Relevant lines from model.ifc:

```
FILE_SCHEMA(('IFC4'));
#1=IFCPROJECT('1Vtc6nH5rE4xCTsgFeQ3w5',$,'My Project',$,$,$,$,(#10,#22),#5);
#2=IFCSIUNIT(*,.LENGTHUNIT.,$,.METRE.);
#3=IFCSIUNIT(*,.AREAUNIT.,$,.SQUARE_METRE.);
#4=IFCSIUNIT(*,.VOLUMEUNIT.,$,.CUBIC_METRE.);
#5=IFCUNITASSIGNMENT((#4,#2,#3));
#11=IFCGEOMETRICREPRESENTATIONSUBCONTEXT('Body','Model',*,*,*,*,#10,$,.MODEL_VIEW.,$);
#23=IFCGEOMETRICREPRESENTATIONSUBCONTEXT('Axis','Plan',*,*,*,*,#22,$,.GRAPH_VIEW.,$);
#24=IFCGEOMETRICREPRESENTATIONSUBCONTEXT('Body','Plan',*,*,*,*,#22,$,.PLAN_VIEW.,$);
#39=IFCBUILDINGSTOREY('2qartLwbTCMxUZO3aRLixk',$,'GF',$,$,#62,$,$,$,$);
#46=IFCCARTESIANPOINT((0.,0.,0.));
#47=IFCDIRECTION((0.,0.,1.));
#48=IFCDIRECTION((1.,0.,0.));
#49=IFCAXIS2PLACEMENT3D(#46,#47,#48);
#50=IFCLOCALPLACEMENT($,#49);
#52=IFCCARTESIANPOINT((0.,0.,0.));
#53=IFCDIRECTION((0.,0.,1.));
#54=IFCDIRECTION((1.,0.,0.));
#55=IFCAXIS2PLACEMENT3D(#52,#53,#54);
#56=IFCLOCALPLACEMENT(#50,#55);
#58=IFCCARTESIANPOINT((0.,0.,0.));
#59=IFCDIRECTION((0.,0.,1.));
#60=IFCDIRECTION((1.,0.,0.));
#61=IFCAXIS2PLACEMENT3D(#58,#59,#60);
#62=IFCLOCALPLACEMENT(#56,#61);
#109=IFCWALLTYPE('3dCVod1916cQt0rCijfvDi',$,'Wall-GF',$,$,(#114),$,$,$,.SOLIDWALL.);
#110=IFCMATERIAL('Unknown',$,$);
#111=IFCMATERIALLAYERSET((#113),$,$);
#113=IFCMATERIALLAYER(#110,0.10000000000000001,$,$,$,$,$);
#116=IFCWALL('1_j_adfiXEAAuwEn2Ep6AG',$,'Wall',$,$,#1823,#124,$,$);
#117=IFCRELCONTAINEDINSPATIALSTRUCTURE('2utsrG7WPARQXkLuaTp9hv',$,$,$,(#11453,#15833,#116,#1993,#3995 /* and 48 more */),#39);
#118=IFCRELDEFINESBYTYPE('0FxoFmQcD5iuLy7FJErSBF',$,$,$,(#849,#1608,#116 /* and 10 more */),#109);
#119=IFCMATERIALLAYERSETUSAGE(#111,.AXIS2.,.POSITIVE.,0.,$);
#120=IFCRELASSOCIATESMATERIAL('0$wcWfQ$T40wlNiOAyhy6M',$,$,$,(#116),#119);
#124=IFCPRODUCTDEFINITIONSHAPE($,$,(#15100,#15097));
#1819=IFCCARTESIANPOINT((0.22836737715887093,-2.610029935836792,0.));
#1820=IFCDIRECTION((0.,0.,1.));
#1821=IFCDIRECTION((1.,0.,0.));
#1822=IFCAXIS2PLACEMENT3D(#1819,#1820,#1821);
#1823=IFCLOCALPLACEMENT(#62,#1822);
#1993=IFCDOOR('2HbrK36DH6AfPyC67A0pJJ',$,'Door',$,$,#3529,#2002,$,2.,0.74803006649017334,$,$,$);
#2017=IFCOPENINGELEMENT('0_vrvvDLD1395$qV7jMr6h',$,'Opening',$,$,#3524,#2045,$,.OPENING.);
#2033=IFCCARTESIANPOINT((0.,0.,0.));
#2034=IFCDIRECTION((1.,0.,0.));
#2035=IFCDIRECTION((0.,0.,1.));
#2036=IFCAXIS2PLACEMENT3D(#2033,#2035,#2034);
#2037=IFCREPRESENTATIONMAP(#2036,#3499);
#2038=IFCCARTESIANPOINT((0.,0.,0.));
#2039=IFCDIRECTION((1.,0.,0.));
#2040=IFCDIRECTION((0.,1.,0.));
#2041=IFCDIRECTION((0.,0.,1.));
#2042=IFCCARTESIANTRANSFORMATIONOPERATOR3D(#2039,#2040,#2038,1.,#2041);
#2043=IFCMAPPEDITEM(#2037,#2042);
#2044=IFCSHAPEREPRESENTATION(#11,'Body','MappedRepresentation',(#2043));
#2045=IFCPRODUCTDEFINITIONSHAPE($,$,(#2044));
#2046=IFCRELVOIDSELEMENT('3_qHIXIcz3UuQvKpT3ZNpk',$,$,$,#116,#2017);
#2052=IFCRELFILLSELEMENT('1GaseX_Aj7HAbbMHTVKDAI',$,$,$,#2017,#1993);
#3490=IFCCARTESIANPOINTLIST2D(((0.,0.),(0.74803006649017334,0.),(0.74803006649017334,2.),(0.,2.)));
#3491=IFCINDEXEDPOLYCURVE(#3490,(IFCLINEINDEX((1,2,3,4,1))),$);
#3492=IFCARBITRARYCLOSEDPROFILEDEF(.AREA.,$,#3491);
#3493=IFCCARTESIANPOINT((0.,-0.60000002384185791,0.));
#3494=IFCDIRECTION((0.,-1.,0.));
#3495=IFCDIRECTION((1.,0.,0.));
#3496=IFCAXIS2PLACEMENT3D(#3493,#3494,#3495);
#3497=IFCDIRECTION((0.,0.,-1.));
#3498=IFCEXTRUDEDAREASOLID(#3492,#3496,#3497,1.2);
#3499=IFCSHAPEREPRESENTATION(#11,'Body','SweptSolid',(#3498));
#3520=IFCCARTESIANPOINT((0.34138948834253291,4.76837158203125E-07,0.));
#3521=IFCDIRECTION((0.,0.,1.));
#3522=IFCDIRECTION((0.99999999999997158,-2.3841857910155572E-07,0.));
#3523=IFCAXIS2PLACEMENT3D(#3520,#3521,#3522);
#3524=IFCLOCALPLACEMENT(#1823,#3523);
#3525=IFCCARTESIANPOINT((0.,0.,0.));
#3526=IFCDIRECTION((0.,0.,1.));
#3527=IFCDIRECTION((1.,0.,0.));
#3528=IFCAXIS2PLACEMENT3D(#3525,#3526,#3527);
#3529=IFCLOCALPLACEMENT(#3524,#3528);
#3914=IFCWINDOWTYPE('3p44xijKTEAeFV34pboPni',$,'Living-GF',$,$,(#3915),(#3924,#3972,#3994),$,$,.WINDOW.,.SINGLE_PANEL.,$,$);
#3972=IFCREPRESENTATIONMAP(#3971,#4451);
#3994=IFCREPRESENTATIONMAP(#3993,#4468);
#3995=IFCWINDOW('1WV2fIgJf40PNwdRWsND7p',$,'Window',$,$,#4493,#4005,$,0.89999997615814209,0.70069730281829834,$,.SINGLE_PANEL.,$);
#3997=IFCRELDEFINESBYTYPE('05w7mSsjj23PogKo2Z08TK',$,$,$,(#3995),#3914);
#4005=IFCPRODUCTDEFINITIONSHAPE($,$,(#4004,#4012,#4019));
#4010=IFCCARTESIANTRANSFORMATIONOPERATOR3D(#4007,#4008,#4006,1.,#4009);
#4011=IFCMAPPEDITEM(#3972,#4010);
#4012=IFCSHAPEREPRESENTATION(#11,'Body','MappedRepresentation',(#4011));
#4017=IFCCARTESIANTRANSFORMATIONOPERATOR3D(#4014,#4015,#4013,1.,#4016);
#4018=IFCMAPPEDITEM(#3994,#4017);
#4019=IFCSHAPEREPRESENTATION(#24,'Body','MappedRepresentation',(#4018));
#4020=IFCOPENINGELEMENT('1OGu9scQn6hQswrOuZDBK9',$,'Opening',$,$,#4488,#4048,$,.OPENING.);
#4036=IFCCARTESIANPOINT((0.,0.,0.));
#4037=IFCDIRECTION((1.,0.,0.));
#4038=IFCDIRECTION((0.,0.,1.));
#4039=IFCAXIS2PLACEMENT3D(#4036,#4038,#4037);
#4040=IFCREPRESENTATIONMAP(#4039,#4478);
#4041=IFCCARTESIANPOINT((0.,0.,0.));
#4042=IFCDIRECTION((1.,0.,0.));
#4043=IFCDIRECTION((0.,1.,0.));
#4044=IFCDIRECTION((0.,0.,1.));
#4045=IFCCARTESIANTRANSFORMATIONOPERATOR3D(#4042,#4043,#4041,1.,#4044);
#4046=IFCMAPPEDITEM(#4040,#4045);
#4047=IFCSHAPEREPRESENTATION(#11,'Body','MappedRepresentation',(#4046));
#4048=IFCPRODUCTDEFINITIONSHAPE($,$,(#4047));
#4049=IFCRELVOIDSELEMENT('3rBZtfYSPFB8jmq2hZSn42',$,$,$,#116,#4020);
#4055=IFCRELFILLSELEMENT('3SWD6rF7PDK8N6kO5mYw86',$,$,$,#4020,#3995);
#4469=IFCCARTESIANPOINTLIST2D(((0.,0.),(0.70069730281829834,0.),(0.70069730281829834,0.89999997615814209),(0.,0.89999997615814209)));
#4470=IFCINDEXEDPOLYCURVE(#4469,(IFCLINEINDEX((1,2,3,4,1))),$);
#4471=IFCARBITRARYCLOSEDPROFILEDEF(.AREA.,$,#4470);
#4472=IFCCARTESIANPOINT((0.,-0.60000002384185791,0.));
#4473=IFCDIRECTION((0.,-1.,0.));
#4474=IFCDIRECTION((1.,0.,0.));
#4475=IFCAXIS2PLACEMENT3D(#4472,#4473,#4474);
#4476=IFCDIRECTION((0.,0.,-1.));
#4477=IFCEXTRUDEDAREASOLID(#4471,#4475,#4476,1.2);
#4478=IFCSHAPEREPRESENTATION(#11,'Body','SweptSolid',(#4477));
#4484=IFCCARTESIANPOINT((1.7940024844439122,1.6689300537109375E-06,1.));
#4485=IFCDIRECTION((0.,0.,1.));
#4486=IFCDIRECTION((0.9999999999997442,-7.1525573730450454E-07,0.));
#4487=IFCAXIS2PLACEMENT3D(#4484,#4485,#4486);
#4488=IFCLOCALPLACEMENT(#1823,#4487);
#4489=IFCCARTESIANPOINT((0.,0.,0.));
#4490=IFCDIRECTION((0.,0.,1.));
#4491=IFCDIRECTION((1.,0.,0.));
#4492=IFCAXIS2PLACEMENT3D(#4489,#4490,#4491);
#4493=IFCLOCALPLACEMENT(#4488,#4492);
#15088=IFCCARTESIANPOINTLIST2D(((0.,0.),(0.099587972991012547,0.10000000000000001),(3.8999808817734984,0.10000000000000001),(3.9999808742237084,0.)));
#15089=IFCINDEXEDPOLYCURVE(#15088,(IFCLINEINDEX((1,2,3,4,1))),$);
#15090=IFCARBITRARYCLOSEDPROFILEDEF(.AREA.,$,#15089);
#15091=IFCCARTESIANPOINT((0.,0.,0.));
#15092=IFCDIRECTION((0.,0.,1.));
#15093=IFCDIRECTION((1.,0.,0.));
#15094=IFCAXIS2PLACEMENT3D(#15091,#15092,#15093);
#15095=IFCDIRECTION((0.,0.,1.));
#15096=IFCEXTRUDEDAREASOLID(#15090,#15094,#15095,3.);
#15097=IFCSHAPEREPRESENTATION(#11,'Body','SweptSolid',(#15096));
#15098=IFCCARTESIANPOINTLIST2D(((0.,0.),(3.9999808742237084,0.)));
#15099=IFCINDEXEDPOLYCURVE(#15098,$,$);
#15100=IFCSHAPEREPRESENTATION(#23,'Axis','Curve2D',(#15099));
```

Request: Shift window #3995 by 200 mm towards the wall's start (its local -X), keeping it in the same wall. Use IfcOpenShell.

```python
import ifcopenshell
import ifcopenshell.api.geometry
import ifcopenshell.util.placement

model = ifcopenshell.open("model.ifc")

window = model.by_guid("1WV2fIgJf40PNwdRWsND7p")
opening = window.FillsVoids[0].RelatingOpeningElement
wall = opening.VoidsElements[0].RelatingBuildingElement

wall_matrix = ifcopenshell.util.placement.get_local_placement(wall.ObjectPlacement)
shift = wall_matrix[:3, 0] * -0.2
before = ifcopenshell.util.placement.get_local_placement(window.ObjectPlacement)[:3, 3].copy()

# The window is placed relative to its opening, so it follows when the opening moves.
matrix = ifcopenshell.util.placement.get_local_placement(opening.ObjectPlacement)
matrix[:3, 3] += shift
ifcopenshell.api.geometry.edit_object_placement(
    model, product=opening, matrix=matrix, is_si=False, should_transform_children=True
)

after = ifcopenshell.util.placement.get_local_placement(window.ObjectPlacement)[:3, 3]
print("window moved by", (after - before).round(3) + 0.0)

model.write("model_edited.ifc")
```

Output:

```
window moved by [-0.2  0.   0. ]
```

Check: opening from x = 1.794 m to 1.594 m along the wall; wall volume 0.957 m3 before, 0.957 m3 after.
